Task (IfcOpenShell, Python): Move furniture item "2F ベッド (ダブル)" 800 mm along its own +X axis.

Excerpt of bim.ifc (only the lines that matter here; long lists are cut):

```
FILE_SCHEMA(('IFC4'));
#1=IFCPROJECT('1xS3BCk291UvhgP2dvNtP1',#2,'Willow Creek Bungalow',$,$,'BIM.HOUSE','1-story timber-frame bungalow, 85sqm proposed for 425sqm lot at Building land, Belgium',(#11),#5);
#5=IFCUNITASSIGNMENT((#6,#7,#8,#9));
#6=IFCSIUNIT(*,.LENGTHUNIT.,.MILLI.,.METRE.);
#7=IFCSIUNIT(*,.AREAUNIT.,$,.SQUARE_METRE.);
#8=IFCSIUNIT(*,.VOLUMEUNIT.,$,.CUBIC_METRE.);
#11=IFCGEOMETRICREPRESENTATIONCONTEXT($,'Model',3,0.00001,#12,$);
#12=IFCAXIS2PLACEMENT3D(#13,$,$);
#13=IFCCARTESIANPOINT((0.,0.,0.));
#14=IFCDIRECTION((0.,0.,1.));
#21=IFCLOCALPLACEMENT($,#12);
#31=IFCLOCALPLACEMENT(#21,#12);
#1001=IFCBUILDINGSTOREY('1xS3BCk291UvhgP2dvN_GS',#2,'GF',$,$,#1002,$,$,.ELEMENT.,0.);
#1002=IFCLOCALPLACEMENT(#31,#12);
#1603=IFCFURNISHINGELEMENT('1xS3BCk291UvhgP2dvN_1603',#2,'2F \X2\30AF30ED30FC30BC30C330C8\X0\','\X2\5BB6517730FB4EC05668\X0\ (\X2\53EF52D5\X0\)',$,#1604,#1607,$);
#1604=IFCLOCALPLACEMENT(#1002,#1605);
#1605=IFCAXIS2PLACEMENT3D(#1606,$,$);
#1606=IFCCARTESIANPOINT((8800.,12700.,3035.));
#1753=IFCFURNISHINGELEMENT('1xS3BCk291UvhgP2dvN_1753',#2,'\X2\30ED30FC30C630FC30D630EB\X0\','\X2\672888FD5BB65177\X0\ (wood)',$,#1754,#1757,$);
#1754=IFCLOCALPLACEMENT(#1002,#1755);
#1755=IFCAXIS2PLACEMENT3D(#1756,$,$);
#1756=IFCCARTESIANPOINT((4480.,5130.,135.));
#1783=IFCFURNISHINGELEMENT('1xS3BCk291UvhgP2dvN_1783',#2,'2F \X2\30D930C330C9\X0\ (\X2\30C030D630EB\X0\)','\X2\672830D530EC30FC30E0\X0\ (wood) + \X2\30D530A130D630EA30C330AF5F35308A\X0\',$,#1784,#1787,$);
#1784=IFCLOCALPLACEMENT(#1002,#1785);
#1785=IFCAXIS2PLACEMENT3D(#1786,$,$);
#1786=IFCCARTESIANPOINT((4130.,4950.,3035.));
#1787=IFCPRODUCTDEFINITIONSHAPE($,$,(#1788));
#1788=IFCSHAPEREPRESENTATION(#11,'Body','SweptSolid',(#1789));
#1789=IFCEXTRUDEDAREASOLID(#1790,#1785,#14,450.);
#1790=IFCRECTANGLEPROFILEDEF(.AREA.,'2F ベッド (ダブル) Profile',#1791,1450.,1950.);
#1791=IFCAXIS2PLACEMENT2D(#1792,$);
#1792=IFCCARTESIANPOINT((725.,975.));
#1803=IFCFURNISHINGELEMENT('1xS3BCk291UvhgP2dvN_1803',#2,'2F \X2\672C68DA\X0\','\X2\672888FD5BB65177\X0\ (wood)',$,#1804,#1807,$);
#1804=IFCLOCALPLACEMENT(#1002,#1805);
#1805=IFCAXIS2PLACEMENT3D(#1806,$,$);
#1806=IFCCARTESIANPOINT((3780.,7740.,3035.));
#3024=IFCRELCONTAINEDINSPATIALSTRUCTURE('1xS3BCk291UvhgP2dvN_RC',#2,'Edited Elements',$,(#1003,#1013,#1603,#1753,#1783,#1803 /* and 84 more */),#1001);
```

```python
import ifcopenshell
import ifcopenshell.api.geometry
import ifcopenshell.util.placement
import ifcopenshell.util.unit

model = ifcopenshell.open("bim.ifc")
unit_scale = ifcopenshell.util.unit.calculate_unit_scale(model)

item = model.by_guid("1xS3BCk291UvhgP2dvN_1783")
matrix = ifcopenshell.util.placement.get_local_placement(item.ObjectPlacement)
matrix[:3, 3] += matrix[:3, 0] * 0.8 / unit_scale
ifcopenshell.api.geometry.edit_object_placement(model, product=item, matrix=matrix, is_si=False)

print(ifcopenshell.util.placement.get_local_placement(item.ObjectPlacement).round(3) + 0.0)

model.write("bim_v2.ifc")
```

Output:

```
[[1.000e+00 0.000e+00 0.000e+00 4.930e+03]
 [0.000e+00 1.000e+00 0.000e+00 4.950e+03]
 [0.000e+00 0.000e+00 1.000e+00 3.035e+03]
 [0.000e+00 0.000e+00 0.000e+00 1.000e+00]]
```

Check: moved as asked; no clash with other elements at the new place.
